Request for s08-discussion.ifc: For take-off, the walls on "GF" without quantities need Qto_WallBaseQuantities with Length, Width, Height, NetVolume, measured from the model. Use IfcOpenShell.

First a look at what the model holds.

```python
import ifcopenshell
import ifcopenshell.util.element
import ifcopenshell.util.unit

model = ifcopenshell.open("s08-discussion.ifc")
print(model.schema)
for unit_type in ("LENGTHUNIT", "AREAUNIT", "VOLUMEUNIT"):
    print(unit_type, ifcopenshell.util.unit.calculate_unit_scale(model, unit_type))
storey = next(s for s in model.by_type("IfcBuildingStorey") if s.Name == "GF")
walls = [e for e in ifcopenshell.util.element.get_decomposition(storey) if e.is_a("IfcWall")]
for e in sorted(walls, key=lambda e: e.id()):
    print(e.id(), e.is_a(), e.Name, list(ifcopenshell.util.element.get_psets(e, qtos_only=True)), sep=" | ")
```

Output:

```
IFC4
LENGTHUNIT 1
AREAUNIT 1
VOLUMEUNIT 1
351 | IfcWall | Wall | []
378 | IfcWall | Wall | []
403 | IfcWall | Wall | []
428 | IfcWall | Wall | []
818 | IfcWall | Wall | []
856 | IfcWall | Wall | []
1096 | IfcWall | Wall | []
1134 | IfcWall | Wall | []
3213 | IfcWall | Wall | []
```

```python
import ifcopenshell
import ifcopenshell.api.pset
import ifcopenshell.geom
import ifcopenshell.util.element
import ifcopenshell.util.shape
import ifcopenshell.util.unit

model = ifcopenshell.open("s08-discussion.ifc")
unit_scale = ifcopenshell.util.unit.calculate_unit_scale(model)
volume_scale = ifcopenshell.util.unit.calculate_unit_scale(model, "VOLUMEUNIT")
settings = ifcopenshell.geom.settings()

storey = next(s for s in model.by_type("IfcBuildingStorey") if s.Name == "GF")
walls = [e for e in ifcopenshell.util.element.get_decomposition(storey) if e.is_a("IfcWall")]

for e in sorted(walls, key=lambda e: e.id()):
    if ifcopenshell.util.element.get_psets(e, qtos_only=True, should_inherit=False):
        continue
    # Geometry comes back in metres, in the element's own axes.
    shape = ifcopenshell.geom.create_shape(settings, e)
    values = {
        "Length": ifcopenshell.util.shape.get_x(shape.geometry) / unit_scale,
        "Width": ifcopenshell.util.shape.get_y(shape.geometry) / unit_scale,
        "Height": ifcopenshell.util.shape.get_z(shape.geometry) / unit_scale,
        "NetVolume": ifcopenshell.util.shape.get_volume(shape.geometry) / volume_scale,
    }
    qto = ifcopenshell.api.pset.add_qto(model, product=e, name="Qto_WallBaseQuantities")
    ifcopenshell.api.pset.edit_qto(model, qto=qto, properties=values)
    print(e.id(), {k: round(v, 3) for k, v in values.items()})

model.write("s08-discussion_edited.ifc")
```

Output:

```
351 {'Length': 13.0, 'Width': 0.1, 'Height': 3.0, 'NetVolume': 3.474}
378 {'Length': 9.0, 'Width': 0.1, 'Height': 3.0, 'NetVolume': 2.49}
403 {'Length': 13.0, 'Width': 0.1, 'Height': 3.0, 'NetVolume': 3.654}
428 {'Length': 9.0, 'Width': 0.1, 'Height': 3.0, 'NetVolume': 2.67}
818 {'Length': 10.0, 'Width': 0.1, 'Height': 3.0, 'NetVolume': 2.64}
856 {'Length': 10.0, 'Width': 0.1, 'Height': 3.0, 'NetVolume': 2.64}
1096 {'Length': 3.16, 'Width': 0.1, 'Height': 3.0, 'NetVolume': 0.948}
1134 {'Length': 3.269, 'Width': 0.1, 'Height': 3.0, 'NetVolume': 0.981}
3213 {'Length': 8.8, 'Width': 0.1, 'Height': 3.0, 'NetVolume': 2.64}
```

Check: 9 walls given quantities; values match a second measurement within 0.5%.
